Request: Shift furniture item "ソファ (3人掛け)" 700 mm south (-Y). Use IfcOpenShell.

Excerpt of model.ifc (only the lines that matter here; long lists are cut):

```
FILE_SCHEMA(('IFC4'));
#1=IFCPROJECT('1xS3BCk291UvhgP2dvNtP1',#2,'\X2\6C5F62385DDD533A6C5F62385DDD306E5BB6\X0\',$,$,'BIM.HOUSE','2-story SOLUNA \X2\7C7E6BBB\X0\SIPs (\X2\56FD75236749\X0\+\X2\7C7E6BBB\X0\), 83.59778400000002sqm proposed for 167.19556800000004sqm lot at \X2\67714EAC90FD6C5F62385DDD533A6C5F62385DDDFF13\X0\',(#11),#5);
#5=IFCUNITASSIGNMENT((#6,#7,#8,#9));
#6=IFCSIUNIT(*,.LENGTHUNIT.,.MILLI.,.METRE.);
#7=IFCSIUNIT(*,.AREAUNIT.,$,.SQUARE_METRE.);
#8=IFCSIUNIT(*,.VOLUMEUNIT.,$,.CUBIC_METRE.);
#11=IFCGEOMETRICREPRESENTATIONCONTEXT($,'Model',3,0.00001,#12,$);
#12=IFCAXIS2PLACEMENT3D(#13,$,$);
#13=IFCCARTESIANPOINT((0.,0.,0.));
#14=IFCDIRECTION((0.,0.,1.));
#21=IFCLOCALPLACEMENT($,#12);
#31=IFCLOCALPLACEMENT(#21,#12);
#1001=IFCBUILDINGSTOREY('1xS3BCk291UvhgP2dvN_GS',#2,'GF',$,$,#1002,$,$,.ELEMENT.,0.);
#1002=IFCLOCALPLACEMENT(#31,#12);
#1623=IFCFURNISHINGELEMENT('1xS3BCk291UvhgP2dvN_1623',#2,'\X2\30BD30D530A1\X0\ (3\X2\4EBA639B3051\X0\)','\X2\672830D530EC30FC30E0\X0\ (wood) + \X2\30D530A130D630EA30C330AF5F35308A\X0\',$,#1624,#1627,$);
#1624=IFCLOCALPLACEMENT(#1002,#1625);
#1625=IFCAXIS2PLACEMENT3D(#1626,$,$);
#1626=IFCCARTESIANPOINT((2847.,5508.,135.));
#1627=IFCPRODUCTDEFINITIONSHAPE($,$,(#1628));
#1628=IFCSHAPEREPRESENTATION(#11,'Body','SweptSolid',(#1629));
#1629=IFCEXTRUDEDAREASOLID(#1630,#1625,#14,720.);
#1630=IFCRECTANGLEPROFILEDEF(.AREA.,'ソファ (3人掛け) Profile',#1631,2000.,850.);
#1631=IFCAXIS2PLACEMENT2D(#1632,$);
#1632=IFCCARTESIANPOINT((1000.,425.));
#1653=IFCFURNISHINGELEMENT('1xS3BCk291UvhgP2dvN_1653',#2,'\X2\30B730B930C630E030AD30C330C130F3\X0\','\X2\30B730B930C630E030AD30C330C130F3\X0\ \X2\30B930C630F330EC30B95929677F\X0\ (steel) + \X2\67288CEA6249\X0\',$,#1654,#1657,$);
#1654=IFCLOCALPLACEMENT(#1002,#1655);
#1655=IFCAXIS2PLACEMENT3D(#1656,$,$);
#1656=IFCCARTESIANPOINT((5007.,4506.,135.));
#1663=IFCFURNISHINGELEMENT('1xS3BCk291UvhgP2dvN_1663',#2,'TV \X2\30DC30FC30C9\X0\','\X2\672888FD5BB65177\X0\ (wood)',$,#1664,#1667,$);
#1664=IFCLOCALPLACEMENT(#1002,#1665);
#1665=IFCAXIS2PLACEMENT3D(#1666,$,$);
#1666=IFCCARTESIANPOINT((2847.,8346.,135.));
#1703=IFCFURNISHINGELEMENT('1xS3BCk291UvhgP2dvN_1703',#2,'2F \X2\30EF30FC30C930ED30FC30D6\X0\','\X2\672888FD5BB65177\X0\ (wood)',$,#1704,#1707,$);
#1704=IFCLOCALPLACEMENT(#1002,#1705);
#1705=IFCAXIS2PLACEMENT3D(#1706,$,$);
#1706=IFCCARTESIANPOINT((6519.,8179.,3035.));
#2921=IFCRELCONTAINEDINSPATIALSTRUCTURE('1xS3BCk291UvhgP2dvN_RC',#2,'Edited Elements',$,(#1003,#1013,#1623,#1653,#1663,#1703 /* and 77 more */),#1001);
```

```python
import ifcopenshell
import ifcopenshell.api.geometry
import ifcopenshell.util.placement
import ifcopenshell.util.unit

model = ifcopenshell.open("model.ifc")
unit_scale = ifcopenshell.util.unit.calculate_unit_scale(model)

item = model.by_id(1623)
matrix = ifcopenshell.util.placement.get_local_placement(item.ObjectPlacement)
matrix[1, 3] -= 0.7 / unit_scale
ifcopenshell.api.geometry.edit_object_placement(model, product=item, matrix=matrix, is_si=False)

print(ifcopenshell.util.placement.get_local_placement(item.ObjectPlacement).round(3) + 0.0)

model.write("model-out.ifc")
```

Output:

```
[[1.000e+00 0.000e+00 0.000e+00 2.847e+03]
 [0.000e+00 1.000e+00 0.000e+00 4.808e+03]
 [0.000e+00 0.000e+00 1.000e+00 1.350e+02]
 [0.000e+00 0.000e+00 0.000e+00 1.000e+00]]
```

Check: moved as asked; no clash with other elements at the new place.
